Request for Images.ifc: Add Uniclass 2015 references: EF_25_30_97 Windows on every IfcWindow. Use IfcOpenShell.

First a look at what the model holds.

```python
import ifcopenshell

model = ifcopenshell.open("Images.ifc")
print(model.schema)
print("classifications:", [c.Name for c in model.by_type("IfcClassification")])
for ifc_class in ("IfcDoor", "IfcRoof", "IfcStair", "IfcWall", "IfcWindow"):
    print(ifc_class, len(model.by_type(ifc_class)))
```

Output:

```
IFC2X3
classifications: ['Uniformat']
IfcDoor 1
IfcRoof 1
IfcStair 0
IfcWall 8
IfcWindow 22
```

```python
import ifcopenshell
import ifcopenshell.api.classification

model = ifcopenshell.open("Images.ifc")

# IFC2X3 requires Source and Edition and has no link from the project to the system.
system = model.create_entity("IfcClassification", Source="NBS", Edition="2015", Name="Uniclass 2015")

codes = {
    "IfcWindow": ("EF_25_30_97", "Windows"),
}
for ifc_class, (code, name) in codes.items():
    products = model.by_type(ifc_class)
    ifcopenshell.api.classification.add_reference(
        model, products=products, classification=system, identification=code, name=name
    )
    print(code, len(products))

model.write("Images-out.ifc")
```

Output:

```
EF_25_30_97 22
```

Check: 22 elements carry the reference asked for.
